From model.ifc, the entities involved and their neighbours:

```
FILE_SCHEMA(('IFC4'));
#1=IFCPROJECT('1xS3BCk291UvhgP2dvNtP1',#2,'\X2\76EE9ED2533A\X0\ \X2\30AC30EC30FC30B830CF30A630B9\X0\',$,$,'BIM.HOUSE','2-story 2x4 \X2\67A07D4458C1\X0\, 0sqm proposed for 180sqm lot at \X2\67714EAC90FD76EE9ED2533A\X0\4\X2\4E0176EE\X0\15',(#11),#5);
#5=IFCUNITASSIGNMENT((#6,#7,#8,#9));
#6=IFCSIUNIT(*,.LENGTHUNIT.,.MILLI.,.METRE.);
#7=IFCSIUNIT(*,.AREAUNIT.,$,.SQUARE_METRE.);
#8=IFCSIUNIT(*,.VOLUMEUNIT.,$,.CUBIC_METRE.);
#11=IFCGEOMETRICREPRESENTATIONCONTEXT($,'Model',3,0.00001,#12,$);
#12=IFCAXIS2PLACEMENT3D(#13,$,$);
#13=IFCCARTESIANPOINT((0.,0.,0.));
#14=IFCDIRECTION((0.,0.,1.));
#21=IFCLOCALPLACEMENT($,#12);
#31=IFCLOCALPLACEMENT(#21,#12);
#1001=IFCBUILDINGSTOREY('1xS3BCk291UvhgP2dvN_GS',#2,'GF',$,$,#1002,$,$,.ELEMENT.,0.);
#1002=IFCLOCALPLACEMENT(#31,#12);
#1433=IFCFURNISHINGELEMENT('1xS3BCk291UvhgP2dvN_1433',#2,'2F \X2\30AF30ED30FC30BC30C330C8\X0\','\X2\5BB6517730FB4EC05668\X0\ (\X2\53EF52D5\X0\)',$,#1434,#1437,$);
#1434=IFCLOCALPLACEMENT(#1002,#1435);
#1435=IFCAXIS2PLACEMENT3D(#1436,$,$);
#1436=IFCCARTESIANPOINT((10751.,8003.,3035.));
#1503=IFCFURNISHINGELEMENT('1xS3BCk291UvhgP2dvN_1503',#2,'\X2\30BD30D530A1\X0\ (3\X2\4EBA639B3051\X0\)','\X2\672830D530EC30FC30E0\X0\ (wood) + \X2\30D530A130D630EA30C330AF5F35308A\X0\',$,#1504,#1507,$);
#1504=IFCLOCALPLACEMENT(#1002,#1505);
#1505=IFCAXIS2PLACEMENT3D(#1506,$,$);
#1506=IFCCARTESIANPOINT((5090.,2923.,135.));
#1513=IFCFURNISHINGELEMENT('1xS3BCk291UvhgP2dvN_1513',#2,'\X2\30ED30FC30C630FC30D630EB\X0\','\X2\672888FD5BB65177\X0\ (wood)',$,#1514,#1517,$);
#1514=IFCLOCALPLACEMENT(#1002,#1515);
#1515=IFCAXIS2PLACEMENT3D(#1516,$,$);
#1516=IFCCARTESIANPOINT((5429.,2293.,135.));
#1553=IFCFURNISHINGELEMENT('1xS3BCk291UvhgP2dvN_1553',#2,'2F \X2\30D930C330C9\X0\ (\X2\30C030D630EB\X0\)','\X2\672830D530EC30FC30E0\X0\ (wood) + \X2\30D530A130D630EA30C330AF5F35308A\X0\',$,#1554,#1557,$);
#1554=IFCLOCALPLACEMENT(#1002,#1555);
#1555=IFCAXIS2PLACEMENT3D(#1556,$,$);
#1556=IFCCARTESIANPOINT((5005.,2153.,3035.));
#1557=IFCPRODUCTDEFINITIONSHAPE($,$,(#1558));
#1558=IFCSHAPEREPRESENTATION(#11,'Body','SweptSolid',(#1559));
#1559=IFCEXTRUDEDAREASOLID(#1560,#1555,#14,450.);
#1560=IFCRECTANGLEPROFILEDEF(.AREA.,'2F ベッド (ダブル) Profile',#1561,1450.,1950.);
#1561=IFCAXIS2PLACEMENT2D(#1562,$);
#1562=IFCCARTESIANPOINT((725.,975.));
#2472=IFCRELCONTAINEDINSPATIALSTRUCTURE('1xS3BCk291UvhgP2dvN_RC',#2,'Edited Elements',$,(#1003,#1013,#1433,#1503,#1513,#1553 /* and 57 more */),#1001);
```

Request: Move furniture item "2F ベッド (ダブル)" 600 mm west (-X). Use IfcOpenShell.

```python
import ifcopenshell
import ifcopenshell.api.geometry
import ifcopenshell.util.placement

model = ifcopenshell.open("model.ifc")

item = model.by_guid("1xS3BCk291UvhgP2dvN_1553")
matrix = ifcopenshell.util.placement.get_local_placement(item.ObjectPlacement)
matrix[0, 3] -= 600.0
ifcopenshell.api.geometry.edit_object_placement(model, product=item, matrix=matrix, is_si=False)

print(ifcopenshell.util.placement.get_local_placement(item.ObjectPlacement).round(3) + 0.0)

model.write("model_v2.ifc")
```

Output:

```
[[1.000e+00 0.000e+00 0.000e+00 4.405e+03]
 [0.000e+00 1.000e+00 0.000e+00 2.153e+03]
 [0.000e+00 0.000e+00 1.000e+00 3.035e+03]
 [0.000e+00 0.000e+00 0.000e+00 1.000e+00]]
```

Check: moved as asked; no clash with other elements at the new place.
